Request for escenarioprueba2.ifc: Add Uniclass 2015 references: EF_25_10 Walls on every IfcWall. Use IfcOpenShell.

First a look at what the model holds.

```python
import ifcopenshell

model = ifcopenshell.open("escenarioprueba2.ifc")
print(model.schema)
print("classifications:", [c.Name for c in model.by_type("IfcClassification")])
for ifc_class in ("IfcDoor", "IfcRoof", "IfcStair", "IfcWall", "IfcWindow"):
    print(ifc_class, len(model.by_type(ifc_class)))
```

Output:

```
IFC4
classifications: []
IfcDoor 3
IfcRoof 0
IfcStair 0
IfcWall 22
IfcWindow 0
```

```python
import ifcopenshell
import ifcopenshell.api.classification

model = ifcopenshell.open("escenarioprueba2.ifc")

system = ifcopenshell.api.classification.add_classification(model, classification="Uniclass 2015")

codes = {
    "IfcWall": ("EF_25_10", "Walls"),
}
for ifc_class, (code, name) in codes.items():
    products = model.by_type(ifc_class)
    ifcopenshell.api.classification.add_reference(
        model, products=products, classification=system, identification=code, name=name
    )
    print(code, len(products))

model.write("escenarioprueba2_updated.ifc")
```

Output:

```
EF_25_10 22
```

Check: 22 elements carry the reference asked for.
